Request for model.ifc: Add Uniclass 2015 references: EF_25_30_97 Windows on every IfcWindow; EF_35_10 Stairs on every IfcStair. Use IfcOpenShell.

First a look at what the model holds.

```python
import ifcopenshell

model = ifcopenshell.open("model.ifc")
print(model.schema)
print("classifications:", [c.Name for c in model.by_type("IfcClassification")])
for ifc_class in ("IfcDoor", "IfcRoof", "IfcStair", "IfcWall", "IfcWindow"):
    print(ifc_class, len(model.by_type(ifc_class)))
```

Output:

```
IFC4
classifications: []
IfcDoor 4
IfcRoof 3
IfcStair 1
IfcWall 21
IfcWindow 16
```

```python
import ifcopenshell
import ifcopenshell.api.classification

model = ifcopenshell.open("model.ifc")

system = ifcopenshell.api.classification.add_classification(model, classification="Uniclass 2015")

codes = {
    "IfcWindow": ("EF_25_30_97", "Windows"),
    "IfcStair": ("EF_35_10", "Stairs"),
}
for ifc_class, (code, name) in codes.items():
    products = model.by_type(ifc_class)
    ifcopenshell.api.classification.add_reference(
        model, products=products, classification=system, identification=code, name=name
    )
    print(code, len(products))

model.write("model-out.ifc")
```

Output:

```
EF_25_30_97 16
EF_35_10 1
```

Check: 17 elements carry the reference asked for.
